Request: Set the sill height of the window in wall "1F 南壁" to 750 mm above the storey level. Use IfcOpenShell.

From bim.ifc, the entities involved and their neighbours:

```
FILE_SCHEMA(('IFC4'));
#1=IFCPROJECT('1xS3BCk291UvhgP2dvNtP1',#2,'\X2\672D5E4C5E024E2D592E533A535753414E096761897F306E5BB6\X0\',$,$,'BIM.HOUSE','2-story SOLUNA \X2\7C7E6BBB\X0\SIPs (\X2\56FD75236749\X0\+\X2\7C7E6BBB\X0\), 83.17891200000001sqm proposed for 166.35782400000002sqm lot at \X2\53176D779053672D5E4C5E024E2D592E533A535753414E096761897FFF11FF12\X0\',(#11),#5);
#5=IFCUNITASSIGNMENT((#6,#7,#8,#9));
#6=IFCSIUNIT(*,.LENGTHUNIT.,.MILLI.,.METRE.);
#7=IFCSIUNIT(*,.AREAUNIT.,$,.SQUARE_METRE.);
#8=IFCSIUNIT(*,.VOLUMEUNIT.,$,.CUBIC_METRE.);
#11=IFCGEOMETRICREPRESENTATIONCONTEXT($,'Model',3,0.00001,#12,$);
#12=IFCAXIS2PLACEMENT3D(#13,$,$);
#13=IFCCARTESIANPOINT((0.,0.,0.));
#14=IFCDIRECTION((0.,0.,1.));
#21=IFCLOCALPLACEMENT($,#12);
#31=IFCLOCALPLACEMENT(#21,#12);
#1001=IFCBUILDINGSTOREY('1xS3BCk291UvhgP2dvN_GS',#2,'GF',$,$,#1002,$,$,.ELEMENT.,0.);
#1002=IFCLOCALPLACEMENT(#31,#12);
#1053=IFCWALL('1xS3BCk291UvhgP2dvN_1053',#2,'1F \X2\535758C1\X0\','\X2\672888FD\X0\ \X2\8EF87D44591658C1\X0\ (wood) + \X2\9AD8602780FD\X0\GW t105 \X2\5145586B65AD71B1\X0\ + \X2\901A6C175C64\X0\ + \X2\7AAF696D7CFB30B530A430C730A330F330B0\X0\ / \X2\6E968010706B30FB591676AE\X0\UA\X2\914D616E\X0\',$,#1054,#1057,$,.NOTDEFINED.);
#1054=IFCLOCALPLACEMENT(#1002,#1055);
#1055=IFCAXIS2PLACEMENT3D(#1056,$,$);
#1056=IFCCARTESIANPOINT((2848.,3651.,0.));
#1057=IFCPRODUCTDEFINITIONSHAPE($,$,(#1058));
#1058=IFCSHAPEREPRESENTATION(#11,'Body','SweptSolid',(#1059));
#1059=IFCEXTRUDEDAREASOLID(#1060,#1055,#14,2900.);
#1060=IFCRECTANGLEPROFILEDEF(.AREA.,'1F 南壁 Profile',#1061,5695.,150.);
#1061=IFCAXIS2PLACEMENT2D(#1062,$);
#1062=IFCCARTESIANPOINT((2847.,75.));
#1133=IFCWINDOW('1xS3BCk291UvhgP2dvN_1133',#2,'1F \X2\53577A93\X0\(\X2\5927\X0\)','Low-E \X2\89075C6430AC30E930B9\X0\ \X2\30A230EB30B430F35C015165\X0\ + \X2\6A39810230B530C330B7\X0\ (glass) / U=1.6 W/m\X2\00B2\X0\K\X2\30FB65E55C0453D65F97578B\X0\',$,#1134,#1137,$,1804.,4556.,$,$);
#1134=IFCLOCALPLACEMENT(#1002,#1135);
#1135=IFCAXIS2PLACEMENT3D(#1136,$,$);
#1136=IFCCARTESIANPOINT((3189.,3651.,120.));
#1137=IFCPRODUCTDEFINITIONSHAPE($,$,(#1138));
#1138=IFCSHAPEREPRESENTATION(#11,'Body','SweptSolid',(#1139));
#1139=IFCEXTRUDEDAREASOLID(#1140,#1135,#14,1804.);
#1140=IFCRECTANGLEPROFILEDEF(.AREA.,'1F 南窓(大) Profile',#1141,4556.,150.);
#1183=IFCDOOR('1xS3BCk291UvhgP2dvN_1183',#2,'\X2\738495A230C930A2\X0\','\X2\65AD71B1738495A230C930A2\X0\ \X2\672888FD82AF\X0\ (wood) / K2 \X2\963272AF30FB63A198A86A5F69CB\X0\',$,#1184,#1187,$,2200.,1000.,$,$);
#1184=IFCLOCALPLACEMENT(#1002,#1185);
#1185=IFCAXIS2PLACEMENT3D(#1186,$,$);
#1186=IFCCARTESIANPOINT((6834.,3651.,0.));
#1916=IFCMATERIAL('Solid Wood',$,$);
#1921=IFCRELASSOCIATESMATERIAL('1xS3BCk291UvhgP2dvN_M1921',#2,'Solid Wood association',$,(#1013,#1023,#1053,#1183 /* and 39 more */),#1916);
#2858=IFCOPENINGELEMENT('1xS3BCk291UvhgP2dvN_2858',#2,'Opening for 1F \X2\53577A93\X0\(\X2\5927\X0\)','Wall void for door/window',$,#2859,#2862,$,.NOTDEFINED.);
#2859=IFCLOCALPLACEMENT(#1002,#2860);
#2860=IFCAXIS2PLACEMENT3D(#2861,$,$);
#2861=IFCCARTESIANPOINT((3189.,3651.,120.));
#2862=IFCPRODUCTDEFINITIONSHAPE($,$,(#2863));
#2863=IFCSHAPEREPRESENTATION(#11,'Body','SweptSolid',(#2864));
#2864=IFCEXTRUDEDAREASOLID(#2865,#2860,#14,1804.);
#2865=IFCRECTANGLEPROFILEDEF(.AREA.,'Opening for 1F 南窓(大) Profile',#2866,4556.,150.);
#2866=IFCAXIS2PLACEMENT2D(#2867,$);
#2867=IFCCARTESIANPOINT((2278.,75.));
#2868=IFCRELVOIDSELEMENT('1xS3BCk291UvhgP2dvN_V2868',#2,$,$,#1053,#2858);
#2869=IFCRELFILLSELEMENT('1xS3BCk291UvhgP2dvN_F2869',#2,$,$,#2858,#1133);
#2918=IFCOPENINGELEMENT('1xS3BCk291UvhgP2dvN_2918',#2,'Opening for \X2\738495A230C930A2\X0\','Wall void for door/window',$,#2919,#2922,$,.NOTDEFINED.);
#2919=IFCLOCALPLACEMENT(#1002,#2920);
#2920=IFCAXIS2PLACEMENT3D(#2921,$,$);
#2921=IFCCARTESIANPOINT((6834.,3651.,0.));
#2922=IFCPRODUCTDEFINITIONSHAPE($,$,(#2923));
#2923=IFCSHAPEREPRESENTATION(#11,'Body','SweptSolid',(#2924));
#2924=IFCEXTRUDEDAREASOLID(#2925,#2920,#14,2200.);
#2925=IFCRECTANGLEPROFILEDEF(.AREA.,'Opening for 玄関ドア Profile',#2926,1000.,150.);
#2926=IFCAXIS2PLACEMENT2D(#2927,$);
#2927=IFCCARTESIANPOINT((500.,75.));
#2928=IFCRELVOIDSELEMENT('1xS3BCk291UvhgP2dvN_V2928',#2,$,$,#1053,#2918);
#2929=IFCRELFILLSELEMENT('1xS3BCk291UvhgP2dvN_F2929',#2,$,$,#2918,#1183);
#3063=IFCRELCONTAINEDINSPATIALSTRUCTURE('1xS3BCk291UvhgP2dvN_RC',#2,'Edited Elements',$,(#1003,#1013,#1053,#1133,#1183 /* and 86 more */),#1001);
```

```python
import numpy as np
import ifcopenshell
import ifcopenshell.api.geometry
import ifcopenshell.geom
import ifcopenshell.util.element
import ifcopenshell.util.placement
import ifcopenshell.util.shape
import ifcopenshell.util.unit

model = ifcopenshell.open("bim.ifc")
unit_scale = ifcopenshell.util.unit.calculate_unit_scale(model)

window = model.by_guid("1xS3BCk291UvhgP2dvN_1133")
opening = window.FillsVoids[0].RelatingOpeningElement
storey = ifcopenshell.util.element.get_container(window, ifc_class="IfcBuildingStorey")
level = ifcopenshell.util.placement.get_local_placement(storey.ObjectPlacement)[2, 3]

# The opening's origin need not be at the sill, so measure its lowest point.
shape = ifcopenshell.geom.create_shape(ifcopenshell.geom.settings(), opening)
bottom = ifcopenshell.util.shape.get_shape_bottom_elevation(shape, shape.geometry) / unit_scale
dz = level + 750.0 - bottom

shift = np.array([0.0, 0.0, dz])
# The window is not placed relative to its opening, so move both.
for product in (opening, window):
    matrix = ifcopenshell.util.placement.get_local_placement(product.ObjectPlacement)
    matrix[:3, 3] += shift
    ifcopenshell.api.geometry.edit_object_placement(model, product=product, matrix=matrix, is_si=False)

print(f"moved by {dz * unit_scale:+.3f} m")

model.write("bim-out.ifc")
```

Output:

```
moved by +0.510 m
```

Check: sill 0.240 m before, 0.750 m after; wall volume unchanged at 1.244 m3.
